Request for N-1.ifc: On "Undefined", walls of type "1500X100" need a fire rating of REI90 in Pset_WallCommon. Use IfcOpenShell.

First a look at what the model holds.

```python
import ifcopenshell
import ifcopenshell.util.element

model = ifcopenshell.open("N-1.ifc")
print(model.schema)
storey = next(s for s in model.by_type("IfcBuildingStorey") if s.Name == "Undefined")
walls = [e for e in ifcopenshell.util.element.get_decomposition(storey) if e.is_a("IfcWall")]
seen = {}
for e in walls:
    element_type = ifcopenshell.util.element.get_type(e)
    key = (element_type.Name if element_type != e and element_type else None, ifcopenshell.util.element.get_pset(e, "Pset_WallCommon", "FireRating"))
    seen[key] = seen.get(key, 0) + 1
for (name, value), count in sorted(seen.items(), key=str):
    print(count, "x", name, "|", value)
```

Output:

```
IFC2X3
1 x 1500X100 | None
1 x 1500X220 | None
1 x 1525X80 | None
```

```python
import ifcopenshell
import ifcopenshell.api.pset
import ifcopenshell.util.element

model = ifcopenshell.open("N-1.ifc")

storey = next(s for s in model.by_type("IfcBuildingStorey") if s.Name == "Undefined")
walls = [e for e in ifcopenshell.util.element.get_decomposition(storey) if e.is_a("IfcWall")]

count = 0
for e in walls:
    element_type = ifcopenshell.util.element.get_type(e)
    if element_type in (None, e) or element_type.Name != "1500X100":
        continue
    # add_pset returns the element's existing set when there is one.
    pset = ifcopenshell.api.pset.add_pset(model, product=e, name="Pset_WallCommon")
    ifcopenshell.api.pset.edit_pset(model, pset=pset, properties={"FireRating": "REI90"})
    count += 1

print(count, "walls updated")

model.write("N-1_edited.ifc")
```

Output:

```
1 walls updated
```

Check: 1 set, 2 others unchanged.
